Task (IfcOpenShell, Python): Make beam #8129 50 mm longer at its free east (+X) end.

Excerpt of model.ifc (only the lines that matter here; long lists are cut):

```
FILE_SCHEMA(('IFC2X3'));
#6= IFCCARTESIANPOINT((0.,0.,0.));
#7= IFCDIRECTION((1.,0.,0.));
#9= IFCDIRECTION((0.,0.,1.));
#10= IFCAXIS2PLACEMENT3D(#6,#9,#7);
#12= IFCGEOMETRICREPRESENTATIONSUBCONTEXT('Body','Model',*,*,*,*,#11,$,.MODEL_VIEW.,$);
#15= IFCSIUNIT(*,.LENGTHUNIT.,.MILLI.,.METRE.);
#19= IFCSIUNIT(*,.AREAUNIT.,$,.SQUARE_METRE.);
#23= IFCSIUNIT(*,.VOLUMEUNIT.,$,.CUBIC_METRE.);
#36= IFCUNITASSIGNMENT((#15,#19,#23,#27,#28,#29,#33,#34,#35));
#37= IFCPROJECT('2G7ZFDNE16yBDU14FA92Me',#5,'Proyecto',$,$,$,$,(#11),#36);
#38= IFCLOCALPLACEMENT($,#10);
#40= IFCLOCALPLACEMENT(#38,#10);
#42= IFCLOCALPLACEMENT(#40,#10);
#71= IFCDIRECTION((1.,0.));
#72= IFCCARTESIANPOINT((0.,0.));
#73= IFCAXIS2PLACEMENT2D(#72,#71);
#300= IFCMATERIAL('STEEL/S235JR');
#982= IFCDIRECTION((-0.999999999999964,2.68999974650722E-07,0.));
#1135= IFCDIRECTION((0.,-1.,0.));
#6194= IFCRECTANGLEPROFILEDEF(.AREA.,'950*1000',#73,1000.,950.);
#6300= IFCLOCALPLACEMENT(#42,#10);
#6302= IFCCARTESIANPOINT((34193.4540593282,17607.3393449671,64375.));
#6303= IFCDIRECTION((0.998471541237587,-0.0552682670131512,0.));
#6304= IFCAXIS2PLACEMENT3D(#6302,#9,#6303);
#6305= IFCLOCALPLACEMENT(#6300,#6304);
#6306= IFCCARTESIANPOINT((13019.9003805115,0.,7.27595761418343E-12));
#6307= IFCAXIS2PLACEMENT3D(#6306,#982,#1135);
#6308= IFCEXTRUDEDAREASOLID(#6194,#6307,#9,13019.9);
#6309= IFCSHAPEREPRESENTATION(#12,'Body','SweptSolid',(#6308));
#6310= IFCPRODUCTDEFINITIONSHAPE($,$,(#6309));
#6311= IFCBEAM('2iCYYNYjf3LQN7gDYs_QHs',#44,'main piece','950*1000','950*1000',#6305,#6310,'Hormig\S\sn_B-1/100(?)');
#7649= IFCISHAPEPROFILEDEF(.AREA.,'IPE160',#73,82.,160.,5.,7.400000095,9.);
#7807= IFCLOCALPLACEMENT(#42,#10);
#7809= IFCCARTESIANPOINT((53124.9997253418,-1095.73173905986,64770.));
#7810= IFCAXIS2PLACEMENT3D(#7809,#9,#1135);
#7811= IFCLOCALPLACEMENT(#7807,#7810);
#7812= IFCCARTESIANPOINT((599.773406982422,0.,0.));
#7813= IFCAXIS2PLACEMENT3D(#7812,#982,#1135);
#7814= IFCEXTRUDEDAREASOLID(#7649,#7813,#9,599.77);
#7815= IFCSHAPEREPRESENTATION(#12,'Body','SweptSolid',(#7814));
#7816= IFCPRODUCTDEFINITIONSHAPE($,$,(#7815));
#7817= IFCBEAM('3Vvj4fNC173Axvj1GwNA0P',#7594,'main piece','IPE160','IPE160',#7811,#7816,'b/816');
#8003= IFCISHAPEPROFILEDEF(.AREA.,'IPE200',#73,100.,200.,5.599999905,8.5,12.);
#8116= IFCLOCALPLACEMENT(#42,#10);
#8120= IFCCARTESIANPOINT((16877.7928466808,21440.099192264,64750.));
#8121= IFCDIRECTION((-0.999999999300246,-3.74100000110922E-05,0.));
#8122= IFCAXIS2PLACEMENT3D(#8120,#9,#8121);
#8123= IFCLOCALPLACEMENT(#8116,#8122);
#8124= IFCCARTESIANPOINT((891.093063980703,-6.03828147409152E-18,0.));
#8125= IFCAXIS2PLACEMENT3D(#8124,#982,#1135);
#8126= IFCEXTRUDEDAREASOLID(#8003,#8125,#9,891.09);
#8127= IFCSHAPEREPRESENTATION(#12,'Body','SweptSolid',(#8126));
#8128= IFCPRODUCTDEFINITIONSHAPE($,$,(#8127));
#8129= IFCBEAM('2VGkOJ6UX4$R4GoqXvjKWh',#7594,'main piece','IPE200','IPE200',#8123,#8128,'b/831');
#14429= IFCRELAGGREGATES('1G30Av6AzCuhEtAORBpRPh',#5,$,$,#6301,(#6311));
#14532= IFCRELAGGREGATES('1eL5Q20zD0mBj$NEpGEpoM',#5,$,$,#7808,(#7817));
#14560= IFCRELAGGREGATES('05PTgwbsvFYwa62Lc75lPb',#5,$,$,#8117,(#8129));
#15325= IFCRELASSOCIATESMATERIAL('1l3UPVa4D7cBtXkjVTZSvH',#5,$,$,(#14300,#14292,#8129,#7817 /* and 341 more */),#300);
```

```python
import ifcopenshell
import ifcopenshell.util.representation
import ifcopenshell.util.unit

model = ifcopenshell.open("model.ifc")
unit_scale = ifcopenshell.util.unit.calculate_unit_scale(model)

member = model.by_id(8129)
change = 0.05 / unit_scale

# The extrusion runs towards the end named, so only its depth changes.
body = ifcopenshell.util.representation.get_representation(member, "Model", "Body")
solid = body.Items[0]
old_length = solid.Depth
solid.Depth += change

print(f"length {old_length:g} -> {solid.Depth:g}")

model.write("model_updated.ifc")
```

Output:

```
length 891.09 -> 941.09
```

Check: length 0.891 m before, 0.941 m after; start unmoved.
